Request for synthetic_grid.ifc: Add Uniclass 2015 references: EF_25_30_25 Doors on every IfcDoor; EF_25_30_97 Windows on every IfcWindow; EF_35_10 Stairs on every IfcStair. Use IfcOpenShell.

First a look at what the model holds.

```python
import ifcopenshell

model = ifcopenshell.open("synthetic_grid.ifc")
print(model.schema)
print("classifications:", [c.Name for c in model.by_type("IfcClassification")])
for ifc_class in ("IfcDoor", "IfcRoof", "IfcStair", "IfcWall", "IfcWindow"):
    print(ifc_class, len(model.by_type(ifc_class)))
```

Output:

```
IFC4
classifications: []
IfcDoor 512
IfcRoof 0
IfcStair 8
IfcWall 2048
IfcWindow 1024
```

```python
import ifcopenshell
import ifcopenshell.api.classification

model = ifcopenshell.open("synthetic_grid.ifc")

system = ifcopenshell.api.classification.add_classification(model, classification="Uniclass 2015")

codes = {
    "IfcDoor": ("EF_25_30_25", "Doors"),
    "IfcWindow": ("EF_25_30_97", "Windows"),
    "IfcStair": ("EF_35_10", "Stairs"),
}
for ifc_class, (code, name) in codes.items():
    products = model.by_type(ifc_class)
    ifcopenshell.api.classification.add_reference(
        model, products=products, classification=system, identification=code, name=name
    )
    print(code, len(products))

model.write("synthetic_grid_edited.ifc")
```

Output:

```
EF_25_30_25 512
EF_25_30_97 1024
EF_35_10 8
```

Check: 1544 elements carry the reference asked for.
